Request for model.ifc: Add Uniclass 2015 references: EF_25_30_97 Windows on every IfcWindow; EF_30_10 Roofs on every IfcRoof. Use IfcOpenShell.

First a look at what the model holds.

```python
import ifcopenshell

model = ifcopenshell.open("model.ifc")
print(model.schema)
print("classifications:", [c.Name for c in model.by_type("IfcClassification")])
for ifc_class in ("IfcDoor", "IfcRoof", "IfcStair", "IfcWall", "IfcWindow"):
    print(ifc_class, len(model.by_type(ifc_class)))
```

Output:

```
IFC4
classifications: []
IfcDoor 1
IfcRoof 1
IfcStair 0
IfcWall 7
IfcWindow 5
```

```python
import ifcopenshell
import ifcopenshell.api.classification

model = ifcopenshell.open("model.ifc")

system = ifcopenshell.api.classification.add_classification(model, classification="Uniclass 2015")

codes = {
    "IfcWindow": ("EF_25_30_97", "Windows"),
    "IfcRoof": ("EF_30_10", "Roofs"),
}
for ifc_class, (code, name) in codes.items():
    products = model.by_type(ifc_class)
    ifcopenshell.api.classification.add_reference(
        model, products=products, classification=system, identification=code, name=name
    )
    print(code, len(products))

model.write("model_edited.ifc")
```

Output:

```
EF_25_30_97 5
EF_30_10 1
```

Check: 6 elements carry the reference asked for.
